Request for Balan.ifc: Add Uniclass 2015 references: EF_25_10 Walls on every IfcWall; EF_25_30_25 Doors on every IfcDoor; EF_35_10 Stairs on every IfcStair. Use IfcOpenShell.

First a look at what the model holds.

```python
import ifcopenshell

model = ifcopenshell.open("Balan.ifc")
print(model.schema)
print("classifications:", [c.Name for c in model.by_type("IfcClassification")])
for ifc_class in ("IfcDoor", "IfcRoof", "IfcStair", "IfcWall", "IfcWindow"):
    print(ifc_class, len(model.by_type(ifc_class)))
```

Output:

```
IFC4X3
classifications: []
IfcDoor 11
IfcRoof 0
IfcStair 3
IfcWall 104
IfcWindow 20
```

```python
import ifcopenshell
import ifcopenshell.api.classification

model = ifcopenshell.open("Balan.ifc")

system = ifcopenshell.api.classification.add_classification(model, classification="Uniclass 2015")

codes = {
    "IfcWall": ("EF_25_10", "Walls"),
    "IfcDoor": ("EF_25_30_25", "Doors"),
    "IfcStair": ("EF_35_10", "Stairs"),
}
for ifc_class, (code, name) in codes.items():
    products = model.by_type(ifc_class)
    ifcopenshell.api.classification.add_reference(
        model, products=products, classification=system, identification=code, name=name
    )
    print(code, len(products))

model.write("Balan_v2.ifc")
```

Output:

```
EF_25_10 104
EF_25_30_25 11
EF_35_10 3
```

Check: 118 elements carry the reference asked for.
